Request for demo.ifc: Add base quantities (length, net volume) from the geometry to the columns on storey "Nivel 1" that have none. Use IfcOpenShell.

First a look at what the model holds.

```python
import ifcopenshell
import ifcopenshell.util.element
import ifcopenshell.util.unit

model = ifcopenshell.open("demo.ifc")
print(model.schema)
for unit_type in ("LENGTHUNIT", "AREAUNIT", "VOLUMEUNIT"):
    print(unit_type, ifcopenshell.util.unit.calculate_unit_scale(model, unit_type))
storey = next(s for s in model.by_type("IfcBuildingStorey") if s.Name == "Nivel 1")
columns = [e for e in ifcopenshell.util.element.get_decomposition(storey) if e.is_a("IfcColumn")]
for e in sorted(columns, key=lambda e: e.id()):
    print(e.id(), e.is_a(), e.Name, list(ifcopenshell.util.element.get_psets(e, qtos_only=True)), sep=" | ")
```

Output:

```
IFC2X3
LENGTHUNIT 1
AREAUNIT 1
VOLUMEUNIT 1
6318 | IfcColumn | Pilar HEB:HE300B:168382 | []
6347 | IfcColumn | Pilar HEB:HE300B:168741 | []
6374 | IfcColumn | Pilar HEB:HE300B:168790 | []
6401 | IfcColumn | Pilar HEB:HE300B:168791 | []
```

```python
import ifcopenshell
import ifcopenshell.api.pset
import ifcopenshell.geom
import ifcopenshell.util.element
import ifcopenshell.util.shape
import ifcopenshell.util.unit

model = ifcopenshell.open("demo.ifc")
unit_scale = ifcopenshell.util.unit.calculate_unit_scale(model)
volume_scale = ifcopenshell.util.unit.calculate_unit_scale(model, "VOLUMEUNIT")
settings = ifcopenshell.geom.settings()

storey = next(s for s in model.by_type("IfcBuildingStorey") if s.Name == "Nivel 1")
columns = [e for e in ifcopenshell.util.element.get_decomposition(storey) if e.is_a("IfcColumn")]

for e in sorted(columns, key=lambda e: e.id()):
    if ifcopenshell.util.element.get_psets(e, qtos_only=True, should_inherit=False):
        continue
    # Geometry comes back in metres, in the element's own axes.
    shape = ifcopenshell.geom.create_shape(settings, e)
    values = {
        "Length": ifcopenshell.util.shape.get_z(shape.geometry) / unit_scale,
        "NetVolume": ifcopenshell.util.shape.get_volume(shape.geometry) / volume_scale,
    }
    qto = ifcopenshell.api.pset.add_qto(model, product=e, name="BaseQuantities")
    ifcopenshell.api.pset.edit_qto(model, qto=qto, properties=values)
    print(e.id(), {k: round(v, 3) for k, v in values.items()})

model.write("demo_updated.ifc")
```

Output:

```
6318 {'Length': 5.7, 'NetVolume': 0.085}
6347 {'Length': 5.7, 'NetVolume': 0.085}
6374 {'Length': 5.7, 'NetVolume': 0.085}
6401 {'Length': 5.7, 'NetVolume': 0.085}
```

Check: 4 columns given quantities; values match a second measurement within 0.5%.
